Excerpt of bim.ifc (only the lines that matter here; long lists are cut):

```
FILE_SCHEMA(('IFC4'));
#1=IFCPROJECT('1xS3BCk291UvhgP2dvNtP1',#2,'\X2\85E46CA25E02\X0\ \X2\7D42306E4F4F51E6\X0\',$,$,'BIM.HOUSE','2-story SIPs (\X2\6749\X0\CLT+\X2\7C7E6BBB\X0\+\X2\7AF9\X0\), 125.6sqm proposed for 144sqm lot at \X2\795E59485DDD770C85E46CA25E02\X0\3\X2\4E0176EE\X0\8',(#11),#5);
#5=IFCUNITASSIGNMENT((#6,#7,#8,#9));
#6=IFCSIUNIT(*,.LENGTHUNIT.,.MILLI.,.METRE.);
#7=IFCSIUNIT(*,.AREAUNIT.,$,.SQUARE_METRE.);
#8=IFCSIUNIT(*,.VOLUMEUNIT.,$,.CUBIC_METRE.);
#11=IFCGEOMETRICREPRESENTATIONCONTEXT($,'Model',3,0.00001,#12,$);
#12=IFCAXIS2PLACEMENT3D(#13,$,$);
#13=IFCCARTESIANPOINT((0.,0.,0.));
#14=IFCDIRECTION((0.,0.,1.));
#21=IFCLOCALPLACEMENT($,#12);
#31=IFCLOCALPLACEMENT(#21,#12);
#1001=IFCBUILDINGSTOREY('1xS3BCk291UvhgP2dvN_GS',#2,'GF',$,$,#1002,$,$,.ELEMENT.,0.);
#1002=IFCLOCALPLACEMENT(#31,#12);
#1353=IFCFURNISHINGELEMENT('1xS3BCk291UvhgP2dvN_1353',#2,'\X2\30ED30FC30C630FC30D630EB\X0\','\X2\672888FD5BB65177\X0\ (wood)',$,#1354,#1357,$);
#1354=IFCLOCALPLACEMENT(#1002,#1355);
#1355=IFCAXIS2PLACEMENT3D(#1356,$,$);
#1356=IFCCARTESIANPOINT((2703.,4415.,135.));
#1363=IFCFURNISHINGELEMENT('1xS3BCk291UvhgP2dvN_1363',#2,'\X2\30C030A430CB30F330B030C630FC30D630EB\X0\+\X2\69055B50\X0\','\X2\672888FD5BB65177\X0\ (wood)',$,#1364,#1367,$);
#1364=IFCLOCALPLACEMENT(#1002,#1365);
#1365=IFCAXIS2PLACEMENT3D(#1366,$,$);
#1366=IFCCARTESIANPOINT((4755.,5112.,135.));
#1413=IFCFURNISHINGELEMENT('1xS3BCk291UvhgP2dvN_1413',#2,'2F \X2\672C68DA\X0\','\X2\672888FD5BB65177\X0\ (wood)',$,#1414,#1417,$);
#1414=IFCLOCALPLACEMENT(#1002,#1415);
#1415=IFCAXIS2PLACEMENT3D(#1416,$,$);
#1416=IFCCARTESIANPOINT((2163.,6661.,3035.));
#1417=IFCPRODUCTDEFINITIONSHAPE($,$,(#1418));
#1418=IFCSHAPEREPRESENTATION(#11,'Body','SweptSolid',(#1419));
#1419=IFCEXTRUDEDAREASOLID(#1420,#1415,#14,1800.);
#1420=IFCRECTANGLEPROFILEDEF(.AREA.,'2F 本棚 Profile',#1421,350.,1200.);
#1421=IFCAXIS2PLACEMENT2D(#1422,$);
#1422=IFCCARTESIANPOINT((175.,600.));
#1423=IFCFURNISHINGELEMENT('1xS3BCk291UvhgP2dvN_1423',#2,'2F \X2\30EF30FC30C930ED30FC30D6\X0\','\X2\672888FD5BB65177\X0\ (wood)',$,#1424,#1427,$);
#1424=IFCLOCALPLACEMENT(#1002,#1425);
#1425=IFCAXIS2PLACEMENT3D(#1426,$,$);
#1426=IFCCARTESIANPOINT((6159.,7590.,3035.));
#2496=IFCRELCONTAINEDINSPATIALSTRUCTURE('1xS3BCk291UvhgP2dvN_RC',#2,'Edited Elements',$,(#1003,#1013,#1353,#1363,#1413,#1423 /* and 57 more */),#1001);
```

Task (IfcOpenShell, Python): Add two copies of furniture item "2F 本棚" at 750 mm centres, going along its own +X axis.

```python
import ifcopenshell
import ifcopenshell.api.geometry
import ifcopenshell.api.root
import ifcopenshell.util.element
import ifcopenshell.util.placement
import ifcopenshell.util.unit

model = ifcopenshell.open("bim.ifc")
unit_scale = ifcopenshell.util.unit.calculate_unit_scale(model)


def reuse_history(source, copy):
    """copy_class also copies each property set's owner history, people and application; keep the originals."""
    for rel in copy.IsDefinedBy:
        if rel.is_a("IfcRelDefinesByProperties") and (history := rel.RelatingPropertyDefinition.OwnerHistory):
            rel.RelatingPropertyDefinition.OwnerHistory = source.OwnerHistory
            ifcopenshell.util.element.remove_deep2(model, history)


source = model.by_id(1413)
base = ifcopenshell.util.placement.get_local_placement(source.ObjectPlacement)
step = base[:3, 0] * 0.75 / unit_scale

for i in range(1, 3):
    copy = ifcopenshell.api.root.copy_class(model, product=source)
    copy.Representation = ifcopenshell.util.element.copy_deep(
        model, source.Representation, exclude=["IfcGeometricRepresentationContext", "IfcRepresentationMap"]
    )
    reuse_history(source, copy)
    matrix = base.copy()
    matrix[:3, 3] += i * step
    print("added at", matrix[:3, 3].round(3) + 0.0)
    ifcopenshell.api.geometry.edit_object_placement(model, product=copy, matrix=matrix, is_si=False)

model.write("bim_edited.ifc")
```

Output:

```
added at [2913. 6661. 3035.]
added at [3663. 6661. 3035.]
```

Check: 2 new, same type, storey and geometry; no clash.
